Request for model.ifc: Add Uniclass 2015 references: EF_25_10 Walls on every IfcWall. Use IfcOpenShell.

First a look at what the model holds.

```python
import ifcopenshell

model = ifcopenshell.open("model.ifc")
print(model.schema)
print("classifications:", [c.Name for c in model.by_type("IfcClassification")])
for ifc_class in ("IfcDoor", "IfcRoof", "IfcStair", "IfcWall", "IfcWindow"):
    print(ifc_class, len(model.by_type(ifc_class)))
```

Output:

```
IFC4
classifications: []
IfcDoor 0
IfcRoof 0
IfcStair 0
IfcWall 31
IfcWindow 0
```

```python
import ifcopenshell
import ifcopenshell.api.classification

model = ifcopenshell.open("model.ifc")

system = ifcopenshell.api.classification.add_classification(model, classification="Uniclass 2015")

codes = {
    "IfcWall": ("EF_25_10", "Walls"),
}
for ifc_class, (code, name) in codes.items():
    products = model.by_type(ifc_class)
    ifcopenshell.api.classification.add_reference(
        model, products=products, classification=system, identification=code, name=name
    )
    print(code, len(products))

model.write("model_updated.ifc")
```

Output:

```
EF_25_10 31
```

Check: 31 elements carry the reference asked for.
